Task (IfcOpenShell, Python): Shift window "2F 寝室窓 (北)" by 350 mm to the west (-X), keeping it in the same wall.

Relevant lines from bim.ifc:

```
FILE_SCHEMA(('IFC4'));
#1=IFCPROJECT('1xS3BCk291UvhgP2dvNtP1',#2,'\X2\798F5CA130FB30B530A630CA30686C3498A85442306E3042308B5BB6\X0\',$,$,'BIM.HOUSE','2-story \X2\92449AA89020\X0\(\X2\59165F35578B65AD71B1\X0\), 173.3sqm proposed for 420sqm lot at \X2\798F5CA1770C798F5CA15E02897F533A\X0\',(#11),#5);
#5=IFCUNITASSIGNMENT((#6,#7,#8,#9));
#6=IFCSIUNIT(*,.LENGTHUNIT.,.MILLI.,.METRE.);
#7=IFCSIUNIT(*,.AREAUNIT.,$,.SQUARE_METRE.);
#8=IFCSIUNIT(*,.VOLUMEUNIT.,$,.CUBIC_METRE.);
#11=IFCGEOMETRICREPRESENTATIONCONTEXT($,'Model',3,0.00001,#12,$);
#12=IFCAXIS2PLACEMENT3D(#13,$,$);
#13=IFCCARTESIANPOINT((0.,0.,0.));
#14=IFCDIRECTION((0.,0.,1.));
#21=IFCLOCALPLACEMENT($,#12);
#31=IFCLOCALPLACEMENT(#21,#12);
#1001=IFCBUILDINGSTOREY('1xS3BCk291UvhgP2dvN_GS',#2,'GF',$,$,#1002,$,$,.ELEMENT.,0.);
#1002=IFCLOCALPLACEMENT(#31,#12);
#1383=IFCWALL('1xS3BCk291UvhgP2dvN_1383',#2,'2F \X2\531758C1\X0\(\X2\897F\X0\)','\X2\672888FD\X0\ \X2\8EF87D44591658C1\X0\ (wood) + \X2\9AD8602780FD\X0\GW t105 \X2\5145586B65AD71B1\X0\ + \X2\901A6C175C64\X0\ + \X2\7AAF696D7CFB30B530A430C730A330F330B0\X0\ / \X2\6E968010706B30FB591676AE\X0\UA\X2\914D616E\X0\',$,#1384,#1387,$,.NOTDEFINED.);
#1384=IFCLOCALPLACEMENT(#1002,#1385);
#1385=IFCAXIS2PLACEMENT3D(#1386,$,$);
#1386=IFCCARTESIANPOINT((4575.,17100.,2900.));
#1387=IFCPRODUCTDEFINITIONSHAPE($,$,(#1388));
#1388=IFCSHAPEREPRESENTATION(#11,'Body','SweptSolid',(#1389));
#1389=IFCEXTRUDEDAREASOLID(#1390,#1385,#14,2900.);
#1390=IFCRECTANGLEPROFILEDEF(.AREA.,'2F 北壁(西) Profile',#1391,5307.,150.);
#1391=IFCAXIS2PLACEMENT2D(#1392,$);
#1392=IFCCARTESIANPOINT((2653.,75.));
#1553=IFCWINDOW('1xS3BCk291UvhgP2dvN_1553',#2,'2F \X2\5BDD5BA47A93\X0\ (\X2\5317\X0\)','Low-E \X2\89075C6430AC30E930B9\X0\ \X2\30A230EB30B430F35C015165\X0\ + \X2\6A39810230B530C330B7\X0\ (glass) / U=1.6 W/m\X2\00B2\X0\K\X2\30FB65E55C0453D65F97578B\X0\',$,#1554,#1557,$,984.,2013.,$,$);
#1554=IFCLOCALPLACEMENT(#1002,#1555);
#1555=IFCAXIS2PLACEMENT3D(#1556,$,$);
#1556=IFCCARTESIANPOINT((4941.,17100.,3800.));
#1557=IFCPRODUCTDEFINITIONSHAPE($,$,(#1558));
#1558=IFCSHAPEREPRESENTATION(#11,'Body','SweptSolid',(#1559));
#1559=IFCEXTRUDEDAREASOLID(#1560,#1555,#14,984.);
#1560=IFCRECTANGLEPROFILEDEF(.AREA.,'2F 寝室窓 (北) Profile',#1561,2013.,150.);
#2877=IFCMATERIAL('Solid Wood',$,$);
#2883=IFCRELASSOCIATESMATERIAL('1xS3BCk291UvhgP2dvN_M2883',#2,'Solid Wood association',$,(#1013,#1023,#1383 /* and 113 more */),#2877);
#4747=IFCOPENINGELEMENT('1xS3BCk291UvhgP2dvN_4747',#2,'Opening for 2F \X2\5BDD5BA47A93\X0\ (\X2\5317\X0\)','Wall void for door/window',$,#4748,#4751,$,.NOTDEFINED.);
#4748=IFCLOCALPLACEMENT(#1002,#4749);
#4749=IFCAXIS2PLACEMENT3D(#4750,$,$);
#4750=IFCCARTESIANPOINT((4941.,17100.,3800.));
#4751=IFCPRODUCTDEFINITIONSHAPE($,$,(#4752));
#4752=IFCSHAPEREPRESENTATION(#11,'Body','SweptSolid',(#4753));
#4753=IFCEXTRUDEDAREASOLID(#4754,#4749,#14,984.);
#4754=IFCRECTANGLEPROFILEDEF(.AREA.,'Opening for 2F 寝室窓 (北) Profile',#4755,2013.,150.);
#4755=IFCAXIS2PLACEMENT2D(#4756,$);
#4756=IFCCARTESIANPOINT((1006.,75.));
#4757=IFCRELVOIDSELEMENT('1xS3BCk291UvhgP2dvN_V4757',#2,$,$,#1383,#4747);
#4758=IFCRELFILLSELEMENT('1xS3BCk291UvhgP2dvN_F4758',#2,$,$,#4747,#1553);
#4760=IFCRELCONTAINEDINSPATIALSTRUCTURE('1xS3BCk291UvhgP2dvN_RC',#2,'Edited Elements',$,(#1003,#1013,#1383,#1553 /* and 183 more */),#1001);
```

```python
import ifcopenshell
import ifcopenshell.api.geometry
import ifcopenshell.util.placement
import ifcopenshell.util.unit

model = ifcopenshell.open("bim.ifc")
unit_scale = ifcopenshell.util.unit.calculate_unit_scale(model)

window = model.by_guid("1xS3BCk291UvhgP2dvN_1553")
opening = window.FillsVoids[0].RelatingOpeningElement
wall = opening.VoidsElements[0].RelatingBuildingElement

wall_matrix = ifcopenshell.util.placement.get_local_placement(wall.ObjectPlacement)
shift = wall_matrix[:3, 0] * -0.35 / unit_scale
before = ifcopenshell.util.placement.get_local_placement(window.ObjectPlacement)[:3, 3].copy()

# The window is not placed relative to its opening, so move both.
for product in (opening, window):
    matrix = ifcopenshell.util.placement.get_local_placement(product.ObjectPlacement)
    matrix[:3, 3] += shift
    ifcopenshell.api.geometry.edit_object_placement(model, product=product, matrix=matrix, is_si=False)

after = ifcopenshell.util.placement.get_local_placement(window.ObjectPlacement)[:3, 3]
print("window moved by", (after - before).round(3) + 0.0)

model.write("bim_updated.ifc")
```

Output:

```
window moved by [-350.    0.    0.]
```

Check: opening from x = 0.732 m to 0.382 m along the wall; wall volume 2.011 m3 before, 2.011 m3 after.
